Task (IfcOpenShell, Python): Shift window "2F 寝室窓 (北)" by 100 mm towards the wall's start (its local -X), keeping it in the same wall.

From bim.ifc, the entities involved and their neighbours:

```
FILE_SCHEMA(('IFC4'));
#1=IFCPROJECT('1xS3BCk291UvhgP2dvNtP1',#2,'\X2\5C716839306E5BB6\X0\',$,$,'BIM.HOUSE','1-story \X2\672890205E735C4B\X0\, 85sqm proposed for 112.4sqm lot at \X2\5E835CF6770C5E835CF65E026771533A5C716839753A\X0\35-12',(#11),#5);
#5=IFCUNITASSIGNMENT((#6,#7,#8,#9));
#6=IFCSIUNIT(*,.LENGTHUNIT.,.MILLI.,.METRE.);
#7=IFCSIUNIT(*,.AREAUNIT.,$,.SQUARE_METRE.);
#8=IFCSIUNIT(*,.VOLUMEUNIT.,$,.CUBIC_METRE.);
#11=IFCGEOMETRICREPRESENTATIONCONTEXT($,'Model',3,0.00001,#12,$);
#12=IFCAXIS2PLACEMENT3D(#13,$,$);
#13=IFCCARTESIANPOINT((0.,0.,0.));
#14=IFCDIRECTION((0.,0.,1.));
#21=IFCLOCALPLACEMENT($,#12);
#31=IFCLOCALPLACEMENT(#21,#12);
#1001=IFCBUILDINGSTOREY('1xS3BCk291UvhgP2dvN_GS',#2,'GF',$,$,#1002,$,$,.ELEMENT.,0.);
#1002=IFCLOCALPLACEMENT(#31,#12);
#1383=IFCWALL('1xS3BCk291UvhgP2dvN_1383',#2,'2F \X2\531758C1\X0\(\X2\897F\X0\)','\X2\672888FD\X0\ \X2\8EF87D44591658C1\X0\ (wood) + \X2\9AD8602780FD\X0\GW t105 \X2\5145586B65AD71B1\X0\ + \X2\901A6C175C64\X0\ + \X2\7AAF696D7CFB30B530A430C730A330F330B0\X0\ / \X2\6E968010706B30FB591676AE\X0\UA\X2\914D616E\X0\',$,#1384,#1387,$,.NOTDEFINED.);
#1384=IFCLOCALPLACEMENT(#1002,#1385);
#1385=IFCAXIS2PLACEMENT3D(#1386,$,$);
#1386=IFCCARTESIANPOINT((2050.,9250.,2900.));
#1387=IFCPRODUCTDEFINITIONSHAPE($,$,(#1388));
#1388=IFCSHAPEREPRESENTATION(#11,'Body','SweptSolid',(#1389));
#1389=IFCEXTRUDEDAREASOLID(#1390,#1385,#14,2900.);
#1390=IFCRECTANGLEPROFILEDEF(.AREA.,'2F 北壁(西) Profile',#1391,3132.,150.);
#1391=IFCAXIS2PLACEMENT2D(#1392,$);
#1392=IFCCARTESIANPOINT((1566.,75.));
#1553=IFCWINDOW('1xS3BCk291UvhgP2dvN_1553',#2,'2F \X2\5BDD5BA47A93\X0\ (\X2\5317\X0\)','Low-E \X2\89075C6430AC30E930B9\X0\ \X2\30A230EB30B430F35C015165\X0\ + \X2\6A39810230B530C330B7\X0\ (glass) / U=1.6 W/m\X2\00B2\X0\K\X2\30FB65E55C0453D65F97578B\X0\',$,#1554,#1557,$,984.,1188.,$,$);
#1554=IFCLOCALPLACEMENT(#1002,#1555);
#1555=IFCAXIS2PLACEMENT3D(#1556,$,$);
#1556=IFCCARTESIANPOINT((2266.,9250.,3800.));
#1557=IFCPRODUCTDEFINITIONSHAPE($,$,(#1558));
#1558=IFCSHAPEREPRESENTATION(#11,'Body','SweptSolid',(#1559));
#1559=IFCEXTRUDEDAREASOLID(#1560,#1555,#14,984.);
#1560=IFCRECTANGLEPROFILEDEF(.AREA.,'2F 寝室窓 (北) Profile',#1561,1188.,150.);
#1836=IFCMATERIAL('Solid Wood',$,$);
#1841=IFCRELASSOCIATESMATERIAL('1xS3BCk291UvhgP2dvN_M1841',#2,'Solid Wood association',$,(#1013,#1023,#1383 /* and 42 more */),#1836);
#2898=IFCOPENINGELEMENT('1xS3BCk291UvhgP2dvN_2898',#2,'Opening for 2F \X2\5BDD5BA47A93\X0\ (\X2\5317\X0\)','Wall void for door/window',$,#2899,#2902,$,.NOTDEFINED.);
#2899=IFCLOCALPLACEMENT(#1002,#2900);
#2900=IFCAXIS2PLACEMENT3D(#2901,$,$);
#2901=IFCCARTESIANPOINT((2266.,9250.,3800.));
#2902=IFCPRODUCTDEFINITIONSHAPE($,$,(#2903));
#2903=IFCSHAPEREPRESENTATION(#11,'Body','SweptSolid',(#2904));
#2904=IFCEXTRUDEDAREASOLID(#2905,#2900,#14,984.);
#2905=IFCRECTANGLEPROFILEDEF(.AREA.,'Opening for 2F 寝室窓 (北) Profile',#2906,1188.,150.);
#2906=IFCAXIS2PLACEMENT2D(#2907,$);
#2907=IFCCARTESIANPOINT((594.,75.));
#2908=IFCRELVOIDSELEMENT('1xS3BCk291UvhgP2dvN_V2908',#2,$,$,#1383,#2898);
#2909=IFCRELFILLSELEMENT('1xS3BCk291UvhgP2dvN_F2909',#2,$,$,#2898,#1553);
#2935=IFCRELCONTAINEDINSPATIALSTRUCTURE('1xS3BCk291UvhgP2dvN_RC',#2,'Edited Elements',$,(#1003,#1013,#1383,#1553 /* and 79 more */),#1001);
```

```python
import ifcopenshell
import ifcopenshell.api.geometry
import ifcopenshell.util.placement
import ifcopenshell.util.unit

model = ifcopenshell.open("bim.ifc")
unit_scale = ifcopenshell.util.unit.calculate_unit_scale(model)

window = model.by_id(1553)
opening = window.FillsVoids[0].RelatingOpeningElement
wall = opening.VoidsElements[0].RelatingBuildingElement

wall_matrix = ifcopenshell.util.placement.get_local_placement(wall.ObjectPlacement)
shift = wall_matrix[:3, 0] * -0.1 / unit_scale
before = ifcopenshell.util.placement.get_local_placement(window.ObjectPlacement)[:3, 3].copy()

# The window is not placed relative to its opening, so move both.
for product in (opening, window):
    matrix = ifcopenshell.util.placement.get_local_placement(product.ObjectPlacement)
    matrix[:3, 3] += shift
    ifcopenshell.api.geometry.edit_object_placement(model, product=product, matrix=matrix, is_si=False)

after = ifcopenshell.util.placement.get_local_placement(window.ObjectPlacement)[:3, 3]
print("window moved by", (after - before).round(3) + 0.0)

model.write("bim_rev.ifc")
```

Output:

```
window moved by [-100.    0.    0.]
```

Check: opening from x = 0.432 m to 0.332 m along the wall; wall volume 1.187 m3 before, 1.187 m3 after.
